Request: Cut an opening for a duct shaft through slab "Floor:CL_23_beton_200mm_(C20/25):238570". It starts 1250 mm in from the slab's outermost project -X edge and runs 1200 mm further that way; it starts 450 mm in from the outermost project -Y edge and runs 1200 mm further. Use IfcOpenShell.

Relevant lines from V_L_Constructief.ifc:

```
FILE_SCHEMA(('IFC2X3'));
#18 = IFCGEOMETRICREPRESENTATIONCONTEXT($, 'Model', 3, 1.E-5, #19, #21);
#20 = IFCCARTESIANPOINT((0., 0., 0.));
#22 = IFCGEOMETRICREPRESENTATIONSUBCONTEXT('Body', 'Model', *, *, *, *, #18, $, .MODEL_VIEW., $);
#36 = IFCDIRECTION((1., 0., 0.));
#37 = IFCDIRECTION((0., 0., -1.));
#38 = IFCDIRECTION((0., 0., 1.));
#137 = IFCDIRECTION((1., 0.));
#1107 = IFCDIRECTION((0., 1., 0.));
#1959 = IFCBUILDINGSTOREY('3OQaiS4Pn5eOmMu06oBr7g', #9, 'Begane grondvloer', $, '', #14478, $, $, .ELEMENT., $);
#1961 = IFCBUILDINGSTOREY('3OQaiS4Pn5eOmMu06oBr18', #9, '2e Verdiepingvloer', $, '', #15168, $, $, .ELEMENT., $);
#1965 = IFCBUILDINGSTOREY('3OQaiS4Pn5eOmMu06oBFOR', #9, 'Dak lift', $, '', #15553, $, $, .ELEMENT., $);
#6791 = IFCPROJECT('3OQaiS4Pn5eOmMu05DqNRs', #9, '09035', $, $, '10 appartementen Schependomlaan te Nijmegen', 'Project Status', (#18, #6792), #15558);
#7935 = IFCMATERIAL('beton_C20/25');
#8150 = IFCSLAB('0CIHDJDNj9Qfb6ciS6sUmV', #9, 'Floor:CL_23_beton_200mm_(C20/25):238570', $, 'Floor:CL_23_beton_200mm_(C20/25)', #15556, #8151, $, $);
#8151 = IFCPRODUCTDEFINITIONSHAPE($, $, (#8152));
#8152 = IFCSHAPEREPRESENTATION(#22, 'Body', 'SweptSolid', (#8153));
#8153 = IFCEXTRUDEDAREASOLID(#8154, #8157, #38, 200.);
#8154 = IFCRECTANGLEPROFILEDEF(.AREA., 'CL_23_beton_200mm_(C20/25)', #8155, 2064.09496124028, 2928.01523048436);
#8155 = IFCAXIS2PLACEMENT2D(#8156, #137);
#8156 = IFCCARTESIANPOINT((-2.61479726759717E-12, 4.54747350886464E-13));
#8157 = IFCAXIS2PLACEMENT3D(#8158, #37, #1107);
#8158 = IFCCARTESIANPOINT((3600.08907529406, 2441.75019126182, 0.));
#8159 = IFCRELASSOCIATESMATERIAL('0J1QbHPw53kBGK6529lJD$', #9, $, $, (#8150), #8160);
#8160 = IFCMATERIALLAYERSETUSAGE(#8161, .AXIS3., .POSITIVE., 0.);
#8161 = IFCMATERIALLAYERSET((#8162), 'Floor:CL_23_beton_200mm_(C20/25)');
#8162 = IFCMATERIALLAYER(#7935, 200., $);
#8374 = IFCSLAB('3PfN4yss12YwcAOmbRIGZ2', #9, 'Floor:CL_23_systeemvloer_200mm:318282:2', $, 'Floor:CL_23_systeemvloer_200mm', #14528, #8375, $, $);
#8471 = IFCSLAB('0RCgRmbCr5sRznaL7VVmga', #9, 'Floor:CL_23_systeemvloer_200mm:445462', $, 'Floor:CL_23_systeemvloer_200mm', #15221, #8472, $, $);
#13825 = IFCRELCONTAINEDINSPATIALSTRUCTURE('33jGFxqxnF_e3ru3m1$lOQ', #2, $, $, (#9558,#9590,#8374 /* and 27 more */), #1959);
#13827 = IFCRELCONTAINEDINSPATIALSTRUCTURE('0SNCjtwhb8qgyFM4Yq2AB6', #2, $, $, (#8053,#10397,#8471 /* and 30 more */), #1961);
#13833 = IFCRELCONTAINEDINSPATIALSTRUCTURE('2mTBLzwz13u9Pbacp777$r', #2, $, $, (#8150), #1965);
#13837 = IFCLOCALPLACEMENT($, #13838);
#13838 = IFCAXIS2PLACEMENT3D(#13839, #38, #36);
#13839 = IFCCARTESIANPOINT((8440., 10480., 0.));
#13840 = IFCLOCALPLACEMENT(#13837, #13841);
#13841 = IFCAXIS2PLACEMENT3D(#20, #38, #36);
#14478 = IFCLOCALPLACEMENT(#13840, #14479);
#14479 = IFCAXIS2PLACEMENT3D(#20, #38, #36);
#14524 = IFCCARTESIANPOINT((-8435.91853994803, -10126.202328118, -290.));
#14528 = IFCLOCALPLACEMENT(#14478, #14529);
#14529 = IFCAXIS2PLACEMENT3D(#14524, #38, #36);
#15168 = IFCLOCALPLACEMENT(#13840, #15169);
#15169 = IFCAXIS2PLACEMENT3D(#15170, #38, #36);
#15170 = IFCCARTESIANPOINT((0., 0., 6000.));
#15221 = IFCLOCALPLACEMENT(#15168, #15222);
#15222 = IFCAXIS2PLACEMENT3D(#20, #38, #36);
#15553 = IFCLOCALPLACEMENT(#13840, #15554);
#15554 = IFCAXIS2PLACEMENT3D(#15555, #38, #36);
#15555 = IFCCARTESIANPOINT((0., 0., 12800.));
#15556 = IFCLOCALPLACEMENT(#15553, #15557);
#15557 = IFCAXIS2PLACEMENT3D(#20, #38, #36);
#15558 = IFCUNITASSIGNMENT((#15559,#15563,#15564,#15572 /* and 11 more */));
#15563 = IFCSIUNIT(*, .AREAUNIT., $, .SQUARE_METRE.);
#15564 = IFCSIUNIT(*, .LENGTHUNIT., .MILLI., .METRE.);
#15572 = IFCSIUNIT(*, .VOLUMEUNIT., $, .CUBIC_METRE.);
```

```python
import numpy as np
import ifcopenshell
import ifcopenshell.api.feature
import ifcopenshell.api.geometry
import ifcopenshell.api.root
import ifcopenshell.geom
import ifcopenshell.util.placement
import ifcopenshell.util.representation
import ifcopenshell.util.shape
import ifcopenshell.util.unit

model = ifcopenshell.open("V_L_Constructief.ifc")
unit_scale = ifcopenshell.util.unit.calculate_unit_scale(model)
settings = ifcopenshell.geom.settings()


def volume(element):
    """Net volume in cubic metres, openings subtracted."""
    shape = ifcopenshell.geom.create_shape(settings, element)
    return ifcopenshell.util.shape.get_volume(shape.geometry)


slab = model.by_guid("0CIHDJDNj9Qfb6ciS6sUmV")
before = volume(slab)

# Extent in the slab's own axes, in metres. The edges named are its -X and -Y sides.
slab_shape = ifcopenshell.geom.create_shape(settings, slab)
vertices = ifcopenshell.util.shape.get_vertices(slab_shape.geometry)
x_min, y_min, bottom = vertices.min(axis=0)
top = vertices[:, 2].max()

opening = ifcopenshell.api.root.create_entity(model, ifc_class="IfcOpeningElement", name="Duct shaft opening")
context = ifcopenshell.util.representation.get_context(model, "Model", "Body", "MODEL_VIEW")
width, depth = 1.2, 1.2
outline = [(0.0, 0.0), (width, 0.0), (width, depth), (0.0, depth), (0.0, 0.0)]
# Overshoot both faces by 50 mm so the cut is clean.
shape = ifcopenshell.api.geometry.add_slab_representation(
    model, context=context, depth=top - bottom + 0.1, polyline=outline
)
ifcopenshell.api.geometry.assign_representation(model, product=opening, representation=shape)

matrix = ifcopenshell.util.placement.get_local_placement(slab.ObjectPlacement)
matrix[:, 3] = matrix @ np.append(np.array([x_min + 1.25, y_min + 0.45, bottom - 0.05]) / unit_scale, 1.0)
ifcopenshell.api.geometry.edit_object_placement(model, product=opening, matrix=matrix, is_si=False)
ifcopenshell.api.feature.add_feature(model, feature=opening, element=slab)

after = volume(slab)

print(f"slab volume {before:.3f} -> {after:.3f} m3")

model.write("V_L_Constructief-out.ifc")
```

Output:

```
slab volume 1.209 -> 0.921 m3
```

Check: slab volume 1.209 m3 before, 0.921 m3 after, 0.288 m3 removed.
